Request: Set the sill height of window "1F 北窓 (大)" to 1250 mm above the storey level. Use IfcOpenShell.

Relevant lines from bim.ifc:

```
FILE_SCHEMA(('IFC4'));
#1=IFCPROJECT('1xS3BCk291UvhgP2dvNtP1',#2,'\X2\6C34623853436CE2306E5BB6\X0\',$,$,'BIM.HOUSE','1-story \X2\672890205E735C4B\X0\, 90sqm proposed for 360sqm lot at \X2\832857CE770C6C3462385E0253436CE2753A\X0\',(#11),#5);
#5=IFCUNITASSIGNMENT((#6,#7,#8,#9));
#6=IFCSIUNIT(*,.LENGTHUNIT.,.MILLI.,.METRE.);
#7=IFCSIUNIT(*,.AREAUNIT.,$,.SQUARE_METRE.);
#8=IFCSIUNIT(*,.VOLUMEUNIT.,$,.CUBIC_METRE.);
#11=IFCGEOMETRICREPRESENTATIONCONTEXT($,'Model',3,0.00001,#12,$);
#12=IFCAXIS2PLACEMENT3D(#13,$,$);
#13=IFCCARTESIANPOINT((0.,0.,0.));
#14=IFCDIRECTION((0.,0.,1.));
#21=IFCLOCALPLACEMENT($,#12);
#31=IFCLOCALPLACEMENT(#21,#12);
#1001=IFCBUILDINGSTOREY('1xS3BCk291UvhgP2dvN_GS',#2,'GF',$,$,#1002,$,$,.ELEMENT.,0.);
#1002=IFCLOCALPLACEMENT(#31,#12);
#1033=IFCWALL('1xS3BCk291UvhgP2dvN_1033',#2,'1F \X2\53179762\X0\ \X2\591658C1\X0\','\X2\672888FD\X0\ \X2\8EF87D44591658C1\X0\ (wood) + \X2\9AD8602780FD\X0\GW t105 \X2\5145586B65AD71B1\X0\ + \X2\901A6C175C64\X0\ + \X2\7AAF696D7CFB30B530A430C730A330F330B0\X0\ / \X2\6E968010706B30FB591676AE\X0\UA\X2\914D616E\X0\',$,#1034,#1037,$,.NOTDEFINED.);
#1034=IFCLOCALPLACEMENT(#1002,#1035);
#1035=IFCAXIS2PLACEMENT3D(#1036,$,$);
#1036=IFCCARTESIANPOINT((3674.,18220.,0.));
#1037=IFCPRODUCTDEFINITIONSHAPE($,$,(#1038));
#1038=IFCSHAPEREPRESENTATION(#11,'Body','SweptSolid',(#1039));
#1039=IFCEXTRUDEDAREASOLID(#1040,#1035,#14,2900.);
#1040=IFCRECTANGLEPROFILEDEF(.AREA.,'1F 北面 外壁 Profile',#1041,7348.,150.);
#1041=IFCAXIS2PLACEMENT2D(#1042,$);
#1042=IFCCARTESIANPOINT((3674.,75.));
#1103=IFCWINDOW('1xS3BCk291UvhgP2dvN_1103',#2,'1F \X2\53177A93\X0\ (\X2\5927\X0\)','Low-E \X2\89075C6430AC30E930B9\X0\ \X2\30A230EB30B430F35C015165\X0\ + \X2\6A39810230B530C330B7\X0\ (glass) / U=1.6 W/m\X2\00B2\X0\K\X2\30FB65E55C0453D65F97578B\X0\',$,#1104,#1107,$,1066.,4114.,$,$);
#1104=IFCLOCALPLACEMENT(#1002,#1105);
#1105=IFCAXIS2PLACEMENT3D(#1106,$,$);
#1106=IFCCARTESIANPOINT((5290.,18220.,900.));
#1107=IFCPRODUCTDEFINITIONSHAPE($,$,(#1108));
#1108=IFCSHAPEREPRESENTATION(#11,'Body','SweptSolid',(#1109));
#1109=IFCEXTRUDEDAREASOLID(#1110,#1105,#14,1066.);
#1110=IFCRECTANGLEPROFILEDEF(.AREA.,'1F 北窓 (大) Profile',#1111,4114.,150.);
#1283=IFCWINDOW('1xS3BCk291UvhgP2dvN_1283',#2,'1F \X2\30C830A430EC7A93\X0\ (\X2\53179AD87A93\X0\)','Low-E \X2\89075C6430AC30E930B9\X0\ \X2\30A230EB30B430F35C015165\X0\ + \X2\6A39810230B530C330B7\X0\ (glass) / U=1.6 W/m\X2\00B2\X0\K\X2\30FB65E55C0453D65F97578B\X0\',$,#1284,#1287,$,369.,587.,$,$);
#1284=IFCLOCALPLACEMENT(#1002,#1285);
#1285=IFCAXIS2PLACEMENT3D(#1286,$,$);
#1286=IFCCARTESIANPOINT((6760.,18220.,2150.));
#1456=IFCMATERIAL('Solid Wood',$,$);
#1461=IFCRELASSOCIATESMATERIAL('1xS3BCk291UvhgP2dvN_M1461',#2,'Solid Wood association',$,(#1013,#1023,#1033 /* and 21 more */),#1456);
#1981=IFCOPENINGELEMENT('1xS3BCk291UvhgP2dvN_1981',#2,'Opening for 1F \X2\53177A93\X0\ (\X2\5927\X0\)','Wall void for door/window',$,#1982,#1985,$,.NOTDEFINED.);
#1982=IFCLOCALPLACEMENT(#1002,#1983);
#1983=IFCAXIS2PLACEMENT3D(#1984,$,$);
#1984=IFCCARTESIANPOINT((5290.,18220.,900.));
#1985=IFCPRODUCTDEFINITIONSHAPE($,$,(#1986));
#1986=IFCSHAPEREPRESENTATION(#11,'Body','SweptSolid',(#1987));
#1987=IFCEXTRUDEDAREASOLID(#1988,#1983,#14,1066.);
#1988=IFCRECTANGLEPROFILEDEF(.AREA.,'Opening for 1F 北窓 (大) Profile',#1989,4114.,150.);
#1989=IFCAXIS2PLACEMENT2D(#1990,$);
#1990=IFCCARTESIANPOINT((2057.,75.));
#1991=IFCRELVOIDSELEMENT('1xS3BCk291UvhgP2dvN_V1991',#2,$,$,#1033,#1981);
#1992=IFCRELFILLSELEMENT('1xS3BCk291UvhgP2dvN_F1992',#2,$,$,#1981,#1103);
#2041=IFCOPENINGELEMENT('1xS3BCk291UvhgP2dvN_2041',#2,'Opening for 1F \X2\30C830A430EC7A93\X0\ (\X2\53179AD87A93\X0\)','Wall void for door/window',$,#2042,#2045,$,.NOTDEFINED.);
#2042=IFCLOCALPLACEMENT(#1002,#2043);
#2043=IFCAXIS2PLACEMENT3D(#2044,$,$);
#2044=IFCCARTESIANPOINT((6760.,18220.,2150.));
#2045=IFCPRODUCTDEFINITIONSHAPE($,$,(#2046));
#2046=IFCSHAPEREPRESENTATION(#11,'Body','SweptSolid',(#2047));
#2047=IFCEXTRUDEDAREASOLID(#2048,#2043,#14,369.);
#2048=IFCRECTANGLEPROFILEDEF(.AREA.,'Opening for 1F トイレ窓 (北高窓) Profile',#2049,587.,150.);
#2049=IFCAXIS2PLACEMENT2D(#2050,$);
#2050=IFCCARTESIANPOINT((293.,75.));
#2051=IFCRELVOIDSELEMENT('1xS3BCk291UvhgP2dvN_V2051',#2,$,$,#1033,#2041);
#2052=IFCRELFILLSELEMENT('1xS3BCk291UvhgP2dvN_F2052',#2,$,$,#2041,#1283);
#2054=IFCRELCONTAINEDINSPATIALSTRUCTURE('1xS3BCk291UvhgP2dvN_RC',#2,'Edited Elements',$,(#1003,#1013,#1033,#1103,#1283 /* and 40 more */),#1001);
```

```python
import numpy as np
import ifcopenshell
import ifcopenshell.api.geometry
import ifcopenshell.geom
import ifcopenshell.util.element
import ifcopenshell.util.placement
import ifcopenshell.util.shape
import ifcopenshell.util.unit

model = ifcopenshell.open("bim.ifc")
unit_scale = ifcopenshell.util.unit.calculate_unit_scale(model)

window = model.by_guid("1xS3BCk291UvhgP2dvN_1103")
opening = window.FillsVoids[0].RelatingOpeningElement
storey = ifcopenshell.util.element.get_container(window, ifc_class="IfcBuildingStorey")
level = ifcopenshell.util.placement.get_local_placement(storey.ObjectPlacement)[2, 3]

# The opening's origin need not be at the sill, so measure its lowest point.
shape = ifcopenshell.geom.create_shape(ifcopenshell.geom.settings(), opening)
bottom = ifcopenshell.util.shape.get_shape_bottom_elevation(shape, shape.geometry) / unit_scale
dz = level + 1.25 / unit_scale - bottom

shift = np.array([0.0, 0.0, dz])
# The window is not placed relative to its opening, so move both.
for product in (opening, window):
    matrix = ifcopenshell.util.placement.get_local_placement(product.ObjectPlacement)
    matrix[:3, 3] += shift
    ifcopenshell.api.geometry.edit_object_placement(model, product=product, matrix=matrix, is_si=False)

print(f"moved by {dz * unit_scale:+.3f} m")

model.write("bim_rev.ifc")
```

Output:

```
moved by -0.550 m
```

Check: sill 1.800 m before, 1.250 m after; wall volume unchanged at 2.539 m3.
